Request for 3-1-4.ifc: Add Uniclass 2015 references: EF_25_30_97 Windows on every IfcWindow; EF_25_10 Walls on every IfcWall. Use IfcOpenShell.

First a look at what the model holds.

```python
import ifcopenshell

model = ifcopenshell.open("3-1-4.ifc")
print(model.schema)
print("classifications:", [c.Name for c in model.by_type("IfcClassification")])
for ifc_class in ("IfcDoor", "IfcRoof", "IfcStair", "IfcWall", "IfcWindow"):
    print(ifc_class, len(model.by_type(ifc_class)))
```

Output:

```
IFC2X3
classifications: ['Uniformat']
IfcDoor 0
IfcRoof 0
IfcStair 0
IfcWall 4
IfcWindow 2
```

```python
import ifcopenshell
import ifcopenshell.api.classification

model = ifcopenshell.open("3-1-4.ifc")

# IFC2X3 requires Source and Edition and has no link from the project to the system.
system = model.create_entity("IfcClassification", Source="NBS", Edition="2015", Name="Uniclass 2015")

codes = {
    "IfcWindow": ("EF_25_30_97", "Windows"),
    "IfcWall": ("EF_25_10", "Walls"),
}
for ifc_class, (code, name) in codes.items():
    products = model.by_type(ifc_class)
    ifcopenshell.api.classification.add_reference(
        model, products=products, classification=system, identification=code, name=name
    )
    print(code, len(products))

model.write("3-1-4_updated.ifc")
```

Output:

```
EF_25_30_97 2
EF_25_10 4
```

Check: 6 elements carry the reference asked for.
